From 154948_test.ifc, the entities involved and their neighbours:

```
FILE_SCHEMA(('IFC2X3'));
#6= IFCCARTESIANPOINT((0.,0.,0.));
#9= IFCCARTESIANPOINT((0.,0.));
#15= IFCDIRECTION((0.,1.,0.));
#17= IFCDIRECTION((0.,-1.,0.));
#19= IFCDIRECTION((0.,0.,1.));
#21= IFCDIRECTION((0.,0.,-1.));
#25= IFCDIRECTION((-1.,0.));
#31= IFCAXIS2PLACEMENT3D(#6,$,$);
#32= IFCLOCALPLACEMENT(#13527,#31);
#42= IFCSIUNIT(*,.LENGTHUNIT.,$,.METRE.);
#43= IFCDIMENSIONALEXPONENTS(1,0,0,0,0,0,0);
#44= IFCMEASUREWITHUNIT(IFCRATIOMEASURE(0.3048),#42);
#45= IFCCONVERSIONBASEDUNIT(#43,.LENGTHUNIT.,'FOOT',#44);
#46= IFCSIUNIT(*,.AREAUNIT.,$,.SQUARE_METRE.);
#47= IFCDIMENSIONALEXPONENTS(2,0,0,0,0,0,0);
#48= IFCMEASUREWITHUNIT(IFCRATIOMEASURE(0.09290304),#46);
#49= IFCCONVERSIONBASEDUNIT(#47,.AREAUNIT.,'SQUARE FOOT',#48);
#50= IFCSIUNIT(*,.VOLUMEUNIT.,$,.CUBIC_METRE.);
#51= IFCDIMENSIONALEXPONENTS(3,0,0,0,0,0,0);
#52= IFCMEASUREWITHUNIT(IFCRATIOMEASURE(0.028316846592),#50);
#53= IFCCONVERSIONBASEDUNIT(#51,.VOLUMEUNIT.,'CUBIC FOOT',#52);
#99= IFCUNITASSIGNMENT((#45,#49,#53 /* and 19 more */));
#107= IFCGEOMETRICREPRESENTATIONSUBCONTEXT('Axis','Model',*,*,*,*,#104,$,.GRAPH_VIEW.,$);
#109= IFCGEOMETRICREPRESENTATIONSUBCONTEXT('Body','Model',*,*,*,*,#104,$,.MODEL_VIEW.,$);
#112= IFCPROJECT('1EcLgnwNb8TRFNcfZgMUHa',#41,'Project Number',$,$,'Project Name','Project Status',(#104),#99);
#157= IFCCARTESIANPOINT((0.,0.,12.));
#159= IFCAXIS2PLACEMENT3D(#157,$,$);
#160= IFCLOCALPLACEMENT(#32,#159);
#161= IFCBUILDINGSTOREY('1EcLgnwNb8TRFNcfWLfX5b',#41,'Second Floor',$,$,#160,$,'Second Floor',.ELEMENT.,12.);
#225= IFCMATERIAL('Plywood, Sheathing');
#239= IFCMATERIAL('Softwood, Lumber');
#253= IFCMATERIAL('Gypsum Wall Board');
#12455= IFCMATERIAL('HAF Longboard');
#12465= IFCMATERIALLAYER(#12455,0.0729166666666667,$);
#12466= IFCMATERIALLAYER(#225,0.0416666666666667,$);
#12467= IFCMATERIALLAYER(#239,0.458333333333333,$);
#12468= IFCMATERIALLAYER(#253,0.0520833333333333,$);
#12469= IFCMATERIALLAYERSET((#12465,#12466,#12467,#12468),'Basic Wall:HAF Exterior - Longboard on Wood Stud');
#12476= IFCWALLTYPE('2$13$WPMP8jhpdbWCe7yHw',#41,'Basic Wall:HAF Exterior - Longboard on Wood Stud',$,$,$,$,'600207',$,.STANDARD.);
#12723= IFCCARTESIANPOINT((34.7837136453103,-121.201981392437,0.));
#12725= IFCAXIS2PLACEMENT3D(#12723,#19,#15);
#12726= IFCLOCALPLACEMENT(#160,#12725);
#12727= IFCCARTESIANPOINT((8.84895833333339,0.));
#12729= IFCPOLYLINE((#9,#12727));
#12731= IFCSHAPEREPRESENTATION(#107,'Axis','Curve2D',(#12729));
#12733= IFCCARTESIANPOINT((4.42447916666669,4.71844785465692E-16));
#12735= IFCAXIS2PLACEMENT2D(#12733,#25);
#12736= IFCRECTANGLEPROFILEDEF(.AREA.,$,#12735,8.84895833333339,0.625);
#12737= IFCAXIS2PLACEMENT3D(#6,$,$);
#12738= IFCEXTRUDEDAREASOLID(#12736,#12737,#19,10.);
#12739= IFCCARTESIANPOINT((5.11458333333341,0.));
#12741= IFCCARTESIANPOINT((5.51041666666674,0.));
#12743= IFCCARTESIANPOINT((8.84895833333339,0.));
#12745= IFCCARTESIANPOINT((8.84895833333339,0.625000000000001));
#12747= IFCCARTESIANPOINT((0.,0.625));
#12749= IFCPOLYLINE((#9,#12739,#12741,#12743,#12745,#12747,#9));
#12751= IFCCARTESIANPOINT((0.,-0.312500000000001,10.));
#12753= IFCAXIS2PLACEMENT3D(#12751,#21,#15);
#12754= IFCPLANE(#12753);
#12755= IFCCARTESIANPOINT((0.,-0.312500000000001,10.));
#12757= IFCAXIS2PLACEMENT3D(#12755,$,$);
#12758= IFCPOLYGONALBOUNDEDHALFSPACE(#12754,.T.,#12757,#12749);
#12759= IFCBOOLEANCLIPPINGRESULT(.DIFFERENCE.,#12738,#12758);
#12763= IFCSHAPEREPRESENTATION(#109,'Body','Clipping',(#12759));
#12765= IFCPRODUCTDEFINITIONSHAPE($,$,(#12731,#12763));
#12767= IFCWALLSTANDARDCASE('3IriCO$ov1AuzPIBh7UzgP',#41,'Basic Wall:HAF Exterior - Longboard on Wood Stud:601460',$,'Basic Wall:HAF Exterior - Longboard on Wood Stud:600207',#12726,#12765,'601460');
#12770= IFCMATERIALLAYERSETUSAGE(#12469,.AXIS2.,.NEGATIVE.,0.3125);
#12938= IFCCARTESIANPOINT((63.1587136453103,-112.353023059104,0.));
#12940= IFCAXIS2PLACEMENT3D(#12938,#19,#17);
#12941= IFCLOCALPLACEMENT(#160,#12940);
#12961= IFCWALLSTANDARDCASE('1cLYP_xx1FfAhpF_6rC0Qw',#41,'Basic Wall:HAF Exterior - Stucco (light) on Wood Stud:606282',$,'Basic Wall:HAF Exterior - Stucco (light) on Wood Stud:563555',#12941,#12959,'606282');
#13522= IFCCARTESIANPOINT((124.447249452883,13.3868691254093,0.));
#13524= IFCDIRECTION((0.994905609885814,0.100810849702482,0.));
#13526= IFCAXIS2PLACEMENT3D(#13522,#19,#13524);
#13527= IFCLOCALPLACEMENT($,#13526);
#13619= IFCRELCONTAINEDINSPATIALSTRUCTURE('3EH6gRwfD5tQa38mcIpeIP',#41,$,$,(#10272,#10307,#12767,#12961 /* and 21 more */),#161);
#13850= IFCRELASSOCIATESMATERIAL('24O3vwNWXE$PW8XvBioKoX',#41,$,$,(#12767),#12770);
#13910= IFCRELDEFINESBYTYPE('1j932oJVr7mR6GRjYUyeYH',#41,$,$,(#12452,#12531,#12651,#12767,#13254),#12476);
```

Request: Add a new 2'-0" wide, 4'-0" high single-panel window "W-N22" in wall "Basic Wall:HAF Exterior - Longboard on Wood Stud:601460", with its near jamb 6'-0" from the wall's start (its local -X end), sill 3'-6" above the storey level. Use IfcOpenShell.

```python
import numpy as np
import ifcopenshell
import ifcopenshell.api.feature
import ifcopenshell.api.geometry
import ifcopenshell.api.root
import ifcopenshell.api.spatial
import ifcopenshell.api.type
import ifcopenshell.geom
import ifcopenshell.util.element
import ifcopenshell.util.placement
import ifcopenshell.util.representation
import ifcopenshell.util.shape
import ifcopenshell.util.unit

model = ifcopenshell.open("154948_test.ifc")
unit_scale = ifcopenshell.util.unit.calculate_unit_scale(model)
settings = ifcopenshell.geom.settings()


def volume(element):
    """Net volume in cubic metres, openings subtracted."""
    shape = ifcopenshell.geom.create_shape(settings, element)
    return ifcopenshell.util.shape.get_volume(shape.geometry)


wall = model.by_guid("3IriCO$ov1AuzPIBh7UzgP")
storey = ifcopenshell.util.element.get_container(wall, ifc_class="IfcBuildingStorey")
context = ifcopenshell.util.representation.get_context(model, "Model", "Body", "MODEL_VIEW")
before = volume(wall)

width, height, from_end, sill = 0.6096, 1.2192, 1.8288, 1.0668  # metres

# The wall runs along its own X axis, and the end named is its -X end.
wall_shape = ifcopenshell.geom.create_shape(settings, wall)
x, y, z = ifcopenshell.util.shape.get_vertices(wall_shape.geometry).T
start = x.min() + from_end
face, thickness = float(y.min()), float(y.max() - y.min())
wall_matrix = ifcopenshell.util.placement.get_local_placement(wall.ObjectPlacement)
level = ifcopenshell.util.placement.get_local_placement(storey.ObjectPlacement)[2, 3]


def in_wall(x, y):
    """Placement at x, y metres in the wall's axes, at sill height."""
    matrix = wall_matrix.copy()
    matrix[:, 3] = wall_matrix @ np.array([x / unit_scale, y / unit_scale, 0.0, 1.0])
    matrix[2, 3] = level + sill / unit_scale
    return matrix


# Opening: a box that overshoots both wall faces by 50 mm.
opening = ifcopenshell.api.root.create_entity(model, ifc_class="IfcOpeningElement")
box = ifcopenshell.api.geometry.add_wall_representation(
    model, context=context, length=width, height=height, thickness=thickness + 0.1
)
ifcopenshell.api.geometry.assign_representation(model, product=opening, representation=box)
ifcopenshell.api.geometry.edit_object_placement(model, product=opening, matrix=in_wall(start, face - 0.05), is_si=False)
ifcopenshell.api.feature.add_feature(model, feature=opening, element=wall)

window = ifcopenshell.api.root.create_entity(model, ifc_class="IfcWindow", name="W-N22")
window.OverallWidth, window.OverallHeight = width / unit_scale, height / unit_scale
body = ifcopenshell.api.geometry.add_window_representation(
    model,
    context=context,
    overall_width=window.OverallWidth,
    overall_height=window.OverallHeight,
    partition_type="SINGLE_PANEL",
)
ifcopenshell.api.geometry.assign_representation(model, product=window, representation=body)
ifcopenshell.api.spatial.assign_container(model, products=[window], relating_structure=storey)
fills = ifcopenshell.api.feature.add_filling(model, opening=opening, element=window)
fills.OwnerHistory = window.OwnerHistory  # required in IFC2X3

# IFC2X3 keeps the operation on the window style.
style = ifcopenshell.api.root.create_entity(model, ifc_class="IfcWindowStyle", name="W-N22")
style.OperationType, style.ConstructionType = "SINGLE_PANEL", "NOTDEFINED"
style.ParameterTakesPrecedence = style.Sizeable = False
ifcopenshell.api.type.assign_type(model, related_objects=[window], relating_type=style)

# Centre the window in the wall's thickness.
ifcopenshell.api.geometry.edit_object_placement(model, product=window, matrix=in_wall(start, face), is_si=False)
window_shape = ifcopenshell.geom.create_shape(settings, window)
depth = ifcopenshell.util.shape.get_vertices(window_shape.geometry)[:, 1]
offset = face + thickness / 2 - (depth.min() + depth.max()) / 2
ifcopenshell.api.geometry.edit_object_placement(model, product=window, matrix=in_wall(start, offset), is_si=False)

after = volume(wall)

print(f"wall volume {before:.3f} -> {after:.3f} m3")

model.write("154948_test_rev.ifc")
```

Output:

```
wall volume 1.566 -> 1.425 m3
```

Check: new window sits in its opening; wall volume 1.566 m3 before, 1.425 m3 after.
